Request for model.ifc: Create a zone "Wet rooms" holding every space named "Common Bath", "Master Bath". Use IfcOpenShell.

First a look at what the model holds.

```python
import ifcopenshell

model = ifcopenshell.open("model.ifc")
print(model.schema)
seen = {}
for space in model.by_type("IfcSpace"):
    seen[space.LongName] = seen.get(space.LongName, 0) + 1
for name, count in sorted(seen.items(), key=str):
    print(count, "x", name)
print("zones:", [z.Name for z in model.by_type("IfcZone")][:20])
```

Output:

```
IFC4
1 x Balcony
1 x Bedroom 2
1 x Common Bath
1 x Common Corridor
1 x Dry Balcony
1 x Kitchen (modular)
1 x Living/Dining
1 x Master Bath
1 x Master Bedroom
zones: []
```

```python
import ifcopenshell
import ifcopenshell.api.group
import ifcopenshell.api.root

model = ifcopenshell.open("model.ifc")

names = {"Common Bath", "Master Bath"}
spaces = [s for s in model.by_type("IfcSpace") if s.LongName in names]

zone = ifcopenshell.api.root.create_entity(model, ifc_class="IfcZone", name="Wet rooms")
ifcopenshell.api.group.assign_group(model, products=spaces, group=zone)
print(len(spaces), "spaces in", zone.Name)

model.write("model_edited.ifc")
```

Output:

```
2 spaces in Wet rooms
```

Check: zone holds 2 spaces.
